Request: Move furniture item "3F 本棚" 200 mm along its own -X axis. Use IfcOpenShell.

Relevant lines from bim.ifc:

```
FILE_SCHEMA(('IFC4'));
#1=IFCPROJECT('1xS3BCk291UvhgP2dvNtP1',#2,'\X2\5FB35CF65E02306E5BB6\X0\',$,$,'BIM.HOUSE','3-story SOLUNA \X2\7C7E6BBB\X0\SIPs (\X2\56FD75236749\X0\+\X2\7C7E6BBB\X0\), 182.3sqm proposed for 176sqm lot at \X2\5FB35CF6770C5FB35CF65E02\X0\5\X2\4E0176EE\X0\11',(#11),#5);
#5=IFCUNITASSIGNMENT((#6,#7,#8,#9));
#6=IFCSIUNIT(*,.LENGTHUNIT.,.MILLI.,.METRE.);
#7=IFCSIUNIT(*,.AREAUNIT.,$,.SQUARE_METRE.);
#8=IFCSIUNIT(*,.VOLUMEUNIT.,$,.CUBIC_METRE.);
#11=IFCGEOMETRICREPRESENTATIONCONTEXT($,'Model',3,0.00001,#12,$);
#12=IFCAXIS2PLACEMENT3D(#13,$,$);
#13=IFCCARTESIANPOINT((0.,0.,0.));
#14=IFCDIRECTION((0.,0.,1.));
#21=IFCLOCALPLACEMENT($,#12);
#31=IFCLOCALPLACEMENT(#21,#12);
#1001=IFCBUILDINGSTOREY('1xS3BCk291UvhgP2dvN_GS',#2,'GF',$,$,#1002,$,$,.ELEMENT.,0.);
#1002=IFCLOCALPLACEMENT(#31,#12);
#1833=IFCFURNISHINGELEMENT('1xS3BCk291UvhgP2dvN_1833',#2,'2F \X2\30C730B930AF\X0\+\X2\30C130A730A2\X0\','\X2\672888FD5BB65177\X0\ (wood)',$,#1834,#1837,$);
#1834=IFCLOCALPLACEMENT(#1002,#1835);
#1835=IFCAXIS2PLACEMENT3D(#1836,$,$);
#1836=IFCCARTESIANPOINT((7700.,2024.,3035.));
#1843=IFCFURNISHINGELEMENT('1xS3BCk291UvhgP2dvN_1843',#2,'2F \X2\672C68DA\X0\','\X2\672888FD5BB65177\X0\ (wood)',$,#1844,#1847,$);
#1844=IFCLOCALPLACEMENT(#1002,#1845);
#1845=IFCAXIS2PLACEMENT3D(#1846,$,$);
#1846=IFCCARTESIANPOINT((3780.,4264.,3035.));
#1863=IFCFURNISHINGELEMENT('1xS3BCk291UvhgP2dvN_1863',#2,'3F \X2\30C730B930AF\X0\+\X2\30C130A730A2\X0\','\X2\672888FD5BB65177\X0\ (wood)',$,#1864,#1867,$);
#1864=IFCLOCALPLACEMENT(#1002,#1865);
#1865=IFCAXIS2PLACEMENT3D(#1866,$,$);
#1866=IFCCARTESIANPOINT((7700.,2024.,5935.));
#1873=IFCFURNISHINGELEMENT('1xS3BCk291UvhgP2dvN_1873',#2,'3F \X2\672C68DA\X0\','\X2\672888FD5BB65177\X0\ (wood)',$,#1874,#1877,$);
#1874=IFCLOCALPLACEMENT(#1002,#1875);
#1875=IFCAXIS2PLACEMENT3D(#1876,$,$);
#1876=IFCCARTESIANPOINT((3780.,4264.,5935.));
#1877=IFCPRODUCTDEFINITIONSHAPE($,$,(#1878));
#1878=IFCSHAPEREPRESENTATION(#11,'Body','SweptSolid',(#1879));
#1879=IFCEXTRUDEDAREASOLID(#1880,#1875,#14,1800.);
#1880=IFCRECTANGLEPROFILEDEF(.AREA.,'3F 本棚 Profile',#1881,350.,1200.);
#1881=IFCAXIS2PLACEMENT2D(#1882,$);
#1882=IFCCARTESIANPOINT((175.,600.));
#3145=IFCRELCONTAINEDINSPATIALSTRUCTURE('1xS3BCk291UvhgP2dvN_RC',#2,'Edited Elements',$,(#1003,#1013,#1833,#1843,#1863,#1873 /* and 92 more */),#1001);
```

```python
import ifcopenshell
import ifcopenshell.api.geometry
import ifcopenshell.util.placement
import ifcopenshell.util.unit

model = ifcopenshell.open("bim.ifc")
unit_scale = ifcopenshell.util.unit.calculate_unit_scale(model)

item = model.by_id(1873)
matrix = ifcopenshell.util.placement.get_local_placement(item.ObjectPlacement)
matrix[:3, 3] -= matrix[:3, 0] * 0.2 / unit_scale
ifcopenshell.api.geometry.edit_object_placement(model, product=item, matrix=matrix, is_si=False)

print(ifcopenshell.util.placement.get_local_placement(item.ObjectPlacement).round(3) + 0.0)

model.write("bim_updated.ifc")
```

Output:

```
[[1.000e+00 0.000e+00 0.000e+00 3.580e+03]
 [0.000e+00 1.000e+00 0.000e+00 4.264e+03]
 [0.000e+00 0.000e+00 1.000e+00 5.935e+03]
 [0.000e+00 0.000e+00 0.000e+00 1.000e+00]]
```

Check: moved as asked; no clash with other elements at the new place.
